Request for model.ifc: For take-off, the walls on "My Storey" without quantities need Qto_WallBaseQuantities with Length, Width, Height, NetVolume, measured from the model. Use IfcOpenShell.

First a look at what the model holds.

```python
import ifcopenshell
import ifcopenshell.util.element
import ifcopenshell.util.unit

model = ifcopenshell.open("model.ifc")
print(model.schema)
for unit_type in ("LENGTHUNIT", "AREAUNIT", "VOLUMEUNIT"):
    print(unit_type, ifcopenshell.util.unit.calculate_unit_scale(model, unit_type))
storey = next(s for s in model.by_type("IfcBuildingStorey") if s.Name == "My Storey")
walls = [e for e in ifcopenshell.util.element.get_decomposition(storey) if e.is_a("IfcWall")]
for e in sorted(walls, key=lambda e: e.id()):
    print(e.id(), e.is_a(), e.Name, list(ifcopenshell.util.element.get_psets(e, qtos_only=True)), sep=" | ")
```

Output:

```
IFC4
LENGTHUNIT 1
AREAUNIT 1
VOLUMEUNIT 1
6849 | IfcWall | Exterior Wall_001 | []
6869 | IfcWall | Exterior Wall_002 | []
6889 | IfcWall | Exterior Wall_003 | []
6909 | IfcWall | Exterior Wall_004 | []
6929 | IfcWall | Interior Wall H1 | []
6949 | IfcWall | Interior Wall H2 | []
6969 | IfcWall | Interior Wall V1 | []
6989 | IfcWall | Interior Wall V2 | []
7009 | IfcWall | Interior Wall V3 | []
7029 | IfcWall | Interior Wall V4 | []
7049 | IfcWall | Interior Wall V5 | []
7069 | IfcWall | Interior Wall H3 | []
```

```python
import ifcopenshell
import ifcopenshell.api.pset
import ifcopenshell.geom
import ifcopenshell.util.element
import ifcopenshell.util.shape
import ifcopenshell.util.unit

model = ifcopenshell.open("model.ifc")
unit_scale = ifcopenshell.util.unit.calculate_unit_scale(model)
volume_scale = ifcopenshell.util.unit.calculate_unit_scale(model, "VOLUMEUNIT")
settings = ifcopenshell.geom.settings()

storey = next(s for s in model.by_type("IfcBuildingStorey") if s.Name == "My Storey")
walls = [e for e in ifcopenshell.util.element.get_decomposition(storey) if e.is_a("IfcWall")]

for e in sorted(walls, key=lambda e: e.id()):
    if ifcopenshell.util.element.get_psets(e, qtos_only=True, should_inherit=False):
        continue
    # Geometry comes back in metres, in the element's own axes.
    shape = ifcopenshell.geom.create_shape(settings, e)
    values = {
        "Length": ifcopenshell.util.shape.get_x(shape.geometry) / unit_scale,
        "Width": ifcopenshell.util.shape.get_y(shape.geometry) / unit_scale,
        "Height": ifcopenshell.util.shape.get_z(shape.geometry) / unit_scale,
        "NetVolume": ifcopenshell.util.shape.get_volume(shape.geometry) / volume_scale,
    }
    qto = ifcopenshell.api.pset.add_qto(model, product=e, name="Qto_WallBaseQuantities")
    ifcopenshell.api.pset.edit_qto(model, qto=qto, properties=values)
    print(e.id(), {k: round(v, 3) for k, v in values.items()})

model.write("model_updated.ifc")
```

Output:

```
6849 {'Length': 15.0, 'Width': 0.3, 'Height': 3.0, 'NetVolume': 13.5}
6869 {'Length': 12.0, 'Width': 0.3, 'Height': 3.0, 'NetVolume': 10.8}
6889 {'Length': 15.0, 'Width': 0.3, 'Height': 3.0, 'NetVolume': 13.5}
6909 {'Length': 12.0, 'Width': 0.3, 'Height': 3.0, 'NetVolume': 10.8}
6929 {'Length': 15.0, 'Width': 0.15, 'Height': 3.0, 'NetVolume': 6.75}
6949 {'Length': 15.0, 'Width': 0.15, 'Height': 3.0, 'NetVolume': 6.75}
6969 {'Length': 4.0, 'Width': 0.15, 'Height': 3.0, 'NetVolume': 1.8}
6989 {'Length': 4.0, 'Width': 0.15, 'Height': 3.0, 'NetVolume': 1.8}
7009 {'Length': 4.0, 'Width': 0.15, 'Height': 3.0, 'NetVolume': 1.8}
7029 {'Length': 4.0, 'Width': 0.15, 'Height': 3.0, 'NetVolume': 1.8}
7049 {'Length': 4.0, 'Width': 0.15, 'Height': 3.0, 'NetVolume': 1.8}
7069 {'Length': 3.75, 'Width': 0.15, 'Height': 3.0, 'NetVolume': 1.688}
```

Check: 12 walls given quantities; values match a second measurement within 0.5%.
